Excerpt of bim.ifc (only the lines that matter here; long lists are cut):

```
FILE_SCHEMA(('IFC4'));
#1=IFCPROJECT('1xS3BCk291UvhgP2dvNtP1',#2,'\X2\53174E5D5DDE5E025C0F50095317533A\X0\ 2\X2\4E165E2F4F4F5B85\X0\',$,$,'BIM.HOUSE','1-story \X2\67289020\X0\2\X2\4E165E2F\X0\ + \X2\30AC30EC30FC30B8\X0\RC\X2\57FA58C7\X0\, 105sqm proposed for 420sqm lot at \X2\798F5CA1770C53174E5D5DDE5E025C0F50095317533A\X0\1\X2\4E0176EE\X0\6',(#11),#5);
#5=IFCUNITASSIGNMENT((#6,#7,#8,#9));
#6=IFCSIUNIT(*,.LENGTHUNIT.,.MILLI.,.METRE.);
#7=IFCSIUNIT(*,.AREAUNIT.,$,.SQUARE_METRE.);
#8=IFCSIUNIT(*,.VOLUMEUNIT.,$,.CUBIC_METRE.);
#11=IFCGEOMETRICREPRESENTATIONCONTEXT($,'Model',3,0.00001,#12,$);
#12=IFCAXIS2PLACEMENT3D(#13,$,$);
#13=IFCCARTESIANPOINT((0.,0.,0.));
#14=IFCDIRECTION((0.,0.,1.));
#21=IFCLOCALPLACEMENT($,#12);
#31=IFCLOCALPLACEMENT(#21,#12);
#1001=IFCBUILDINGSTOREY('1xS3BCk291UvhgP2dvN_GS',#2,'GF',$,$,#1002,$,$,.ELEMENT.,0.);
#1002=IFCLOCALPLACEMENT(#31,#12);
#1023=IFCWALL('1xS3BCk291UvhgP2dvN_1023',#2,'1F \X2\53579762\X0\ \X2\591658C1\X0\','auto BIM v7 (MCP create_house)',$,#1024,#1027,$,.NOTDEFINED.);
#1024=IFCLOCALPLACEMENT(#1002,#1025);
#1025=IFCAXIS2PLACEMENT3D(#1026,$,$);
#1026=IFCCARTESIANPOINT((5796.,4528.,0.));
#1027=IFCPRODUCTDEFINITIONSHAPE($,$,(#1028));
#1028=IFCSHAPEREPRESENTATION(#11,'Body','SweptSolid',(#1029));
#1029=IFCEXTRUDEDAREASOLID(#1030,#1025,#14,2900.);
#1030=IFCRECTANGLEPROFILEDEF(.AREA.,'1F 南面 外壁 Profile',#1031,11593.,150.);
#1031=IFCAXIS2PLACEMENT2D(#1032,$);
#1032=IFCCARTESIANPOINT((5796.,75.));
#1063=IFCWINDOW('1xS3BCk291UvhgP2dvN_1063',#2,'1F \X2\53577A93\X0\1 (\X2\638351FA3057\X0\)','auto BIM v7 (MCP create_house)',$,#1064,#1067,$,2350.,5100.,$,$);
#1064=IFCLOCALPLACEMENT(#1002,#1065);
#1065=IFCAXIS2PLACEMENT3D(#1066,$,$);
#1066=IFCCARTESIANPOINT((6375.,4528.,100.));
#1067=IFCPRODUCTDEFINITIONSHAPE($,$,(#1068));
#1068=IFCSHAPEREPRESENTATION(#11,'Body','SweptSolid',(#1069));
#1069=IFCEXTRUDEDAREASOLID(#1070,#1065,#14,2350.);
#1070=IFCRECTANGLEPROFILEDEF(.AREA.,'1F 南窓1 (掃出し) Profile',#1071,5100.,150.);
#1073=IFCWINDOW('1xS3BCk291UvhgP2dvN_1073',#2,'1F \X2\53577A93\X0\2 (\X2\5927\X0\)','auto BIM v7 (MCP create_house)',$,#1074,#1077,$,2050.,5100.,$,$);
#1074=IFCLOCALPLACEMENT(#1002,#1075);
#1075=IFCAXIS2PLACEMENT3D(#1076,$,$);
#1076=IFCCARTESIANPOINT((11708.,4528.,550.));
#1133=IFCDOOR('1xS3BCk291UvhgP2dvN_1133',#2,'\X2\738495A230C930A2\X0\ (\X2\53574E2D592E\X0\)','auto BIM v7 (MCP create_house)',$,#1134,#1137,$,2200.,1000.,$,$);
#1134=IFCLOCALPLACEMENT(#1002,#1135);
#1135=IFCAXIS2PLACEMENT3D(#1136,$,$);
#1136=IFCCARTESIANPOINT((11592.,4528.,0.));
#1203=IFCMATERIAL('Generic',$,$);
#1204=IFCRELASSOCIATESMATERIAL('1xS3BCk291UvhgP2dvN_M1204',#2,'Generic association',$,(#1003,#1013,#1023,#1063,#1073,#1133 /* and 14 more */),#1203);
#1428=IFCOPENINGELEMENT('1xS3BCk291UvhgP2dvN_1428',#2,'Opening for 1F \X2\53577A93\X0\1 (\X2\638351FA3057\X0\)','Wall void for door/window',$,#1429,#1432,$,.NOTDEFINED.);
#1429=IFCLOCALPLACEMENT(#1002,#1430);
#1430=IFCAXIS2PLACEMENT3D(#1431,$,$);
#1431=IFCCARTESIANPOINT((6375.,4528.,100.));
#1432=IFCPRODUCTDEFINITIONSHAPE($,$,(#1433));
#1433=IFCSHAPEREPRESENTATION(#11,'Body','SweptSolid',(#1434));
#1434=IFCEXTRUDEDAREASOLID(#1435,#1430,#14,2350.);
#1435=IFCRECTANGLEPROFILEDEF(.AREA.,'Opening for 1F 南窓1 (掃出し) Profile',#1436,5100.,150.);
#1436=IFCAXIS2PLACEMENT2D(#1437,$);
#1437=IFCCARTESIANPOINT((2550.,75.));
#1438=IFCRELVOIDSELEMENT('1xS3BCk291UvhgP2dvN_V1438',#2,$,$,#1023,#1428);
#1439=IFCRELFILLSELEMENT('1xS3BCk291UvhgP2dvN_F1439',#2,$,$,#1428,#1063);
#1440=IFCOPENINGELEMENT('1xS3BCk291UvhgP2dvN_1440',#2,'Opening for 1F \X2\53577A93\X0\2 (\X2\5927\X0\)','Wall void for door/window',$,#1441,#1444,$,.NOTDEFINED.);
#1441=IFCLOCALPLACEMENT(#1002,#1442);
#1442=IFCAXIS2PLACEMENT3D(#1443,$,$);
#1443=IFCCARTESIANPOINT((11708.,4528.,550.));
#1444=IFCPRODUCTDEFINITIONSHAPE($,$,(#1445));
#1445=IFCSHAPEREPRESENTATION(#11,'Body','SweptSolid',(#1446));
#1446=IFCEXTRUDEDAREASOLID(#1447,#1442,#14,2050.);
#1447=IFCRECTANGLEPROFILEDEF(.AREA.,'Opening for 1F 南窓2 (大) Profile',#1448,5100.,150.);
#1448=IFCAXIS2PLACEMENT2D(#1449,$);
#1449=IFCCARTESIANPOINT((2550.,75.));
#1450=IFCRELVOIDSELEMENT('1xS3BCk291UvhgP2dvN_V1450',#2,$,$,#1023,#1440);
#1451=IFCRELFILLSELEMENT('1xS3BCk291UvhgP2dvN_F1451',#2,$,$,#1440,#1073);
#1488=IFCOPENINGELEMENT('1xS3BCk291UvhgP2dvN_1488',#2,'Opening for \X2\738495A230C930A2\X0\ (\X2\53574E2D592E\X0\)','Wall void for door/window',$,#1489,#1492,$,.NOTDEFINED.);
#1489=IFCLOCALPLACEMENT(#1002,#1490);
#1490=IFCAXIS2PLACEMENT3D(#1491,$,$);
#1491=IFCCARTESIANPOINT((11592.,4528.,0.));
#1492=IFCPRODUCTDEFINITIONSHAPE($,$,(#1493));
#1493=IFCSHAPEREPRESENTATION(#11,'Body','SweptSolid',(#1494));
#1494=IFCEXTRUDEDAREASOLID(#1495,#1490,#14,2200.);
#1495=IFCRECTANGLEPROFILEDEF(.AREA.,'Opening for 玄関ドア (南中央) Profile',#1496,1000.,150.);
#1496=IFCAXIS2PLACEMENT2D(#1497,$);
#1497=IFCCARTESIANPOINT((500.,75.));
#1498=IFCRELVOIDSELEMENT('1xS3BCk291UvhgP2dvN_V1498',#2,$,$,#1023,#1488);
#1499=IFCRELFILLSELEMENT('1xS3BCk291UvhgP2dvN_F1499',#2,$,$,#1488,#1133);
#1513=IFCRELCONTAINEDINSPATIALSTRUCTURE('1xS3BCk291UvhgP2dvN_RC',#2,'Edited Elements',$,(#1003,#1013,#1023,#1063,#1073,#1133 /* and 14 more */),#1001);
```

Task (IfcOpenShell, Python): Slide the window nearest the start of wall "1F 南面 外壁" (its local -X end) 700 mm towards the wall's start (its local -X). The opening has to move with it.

```python
import ifcopenshell
import ifcopenshell.api.geometry
import ifcopenshell.util.placement

model = ifcopenshell.open("bim.ifc")

window = model.by_guid("1xS3BCk291UvhgP2dvN_1063")
opening = window.FillsVoids[0].RelatingOpeningElement
wall = opening.VoidsElements[0].RelatingBuildingElement

wall_matrix = ifcopenshell.util.placement.get_local_placement(wall.ObjectPlacement)
shift = wall_matrix[:3, 0] * -700.0
before = ifcopenshell.util.placement.get_local_placement(window.ObjectPlacement)[:3, 3].copy()

# The window is not placed relative to its opening, so move both.
for product in (opening, window):
    matrix = ifcopenshell.util.placement.get_local_placement(product.ObjectPlacement)
    matrix[:3, 3] += shift
    ifcopenshell.api.geometry.edit_object_placement(model, product=product, matrix=matrix, is_si=False)

after = ifcopenshell.util.placement.get_local_placement(window.ObjectPlacement)[:3, 3]
print("window moved by", (after - before).round(3) + 0.0)

model.write("bim-out.ifc")
```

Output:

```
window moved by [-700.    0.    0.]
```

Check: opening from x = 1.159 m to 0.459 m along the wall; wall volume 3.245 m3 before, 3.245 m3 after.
